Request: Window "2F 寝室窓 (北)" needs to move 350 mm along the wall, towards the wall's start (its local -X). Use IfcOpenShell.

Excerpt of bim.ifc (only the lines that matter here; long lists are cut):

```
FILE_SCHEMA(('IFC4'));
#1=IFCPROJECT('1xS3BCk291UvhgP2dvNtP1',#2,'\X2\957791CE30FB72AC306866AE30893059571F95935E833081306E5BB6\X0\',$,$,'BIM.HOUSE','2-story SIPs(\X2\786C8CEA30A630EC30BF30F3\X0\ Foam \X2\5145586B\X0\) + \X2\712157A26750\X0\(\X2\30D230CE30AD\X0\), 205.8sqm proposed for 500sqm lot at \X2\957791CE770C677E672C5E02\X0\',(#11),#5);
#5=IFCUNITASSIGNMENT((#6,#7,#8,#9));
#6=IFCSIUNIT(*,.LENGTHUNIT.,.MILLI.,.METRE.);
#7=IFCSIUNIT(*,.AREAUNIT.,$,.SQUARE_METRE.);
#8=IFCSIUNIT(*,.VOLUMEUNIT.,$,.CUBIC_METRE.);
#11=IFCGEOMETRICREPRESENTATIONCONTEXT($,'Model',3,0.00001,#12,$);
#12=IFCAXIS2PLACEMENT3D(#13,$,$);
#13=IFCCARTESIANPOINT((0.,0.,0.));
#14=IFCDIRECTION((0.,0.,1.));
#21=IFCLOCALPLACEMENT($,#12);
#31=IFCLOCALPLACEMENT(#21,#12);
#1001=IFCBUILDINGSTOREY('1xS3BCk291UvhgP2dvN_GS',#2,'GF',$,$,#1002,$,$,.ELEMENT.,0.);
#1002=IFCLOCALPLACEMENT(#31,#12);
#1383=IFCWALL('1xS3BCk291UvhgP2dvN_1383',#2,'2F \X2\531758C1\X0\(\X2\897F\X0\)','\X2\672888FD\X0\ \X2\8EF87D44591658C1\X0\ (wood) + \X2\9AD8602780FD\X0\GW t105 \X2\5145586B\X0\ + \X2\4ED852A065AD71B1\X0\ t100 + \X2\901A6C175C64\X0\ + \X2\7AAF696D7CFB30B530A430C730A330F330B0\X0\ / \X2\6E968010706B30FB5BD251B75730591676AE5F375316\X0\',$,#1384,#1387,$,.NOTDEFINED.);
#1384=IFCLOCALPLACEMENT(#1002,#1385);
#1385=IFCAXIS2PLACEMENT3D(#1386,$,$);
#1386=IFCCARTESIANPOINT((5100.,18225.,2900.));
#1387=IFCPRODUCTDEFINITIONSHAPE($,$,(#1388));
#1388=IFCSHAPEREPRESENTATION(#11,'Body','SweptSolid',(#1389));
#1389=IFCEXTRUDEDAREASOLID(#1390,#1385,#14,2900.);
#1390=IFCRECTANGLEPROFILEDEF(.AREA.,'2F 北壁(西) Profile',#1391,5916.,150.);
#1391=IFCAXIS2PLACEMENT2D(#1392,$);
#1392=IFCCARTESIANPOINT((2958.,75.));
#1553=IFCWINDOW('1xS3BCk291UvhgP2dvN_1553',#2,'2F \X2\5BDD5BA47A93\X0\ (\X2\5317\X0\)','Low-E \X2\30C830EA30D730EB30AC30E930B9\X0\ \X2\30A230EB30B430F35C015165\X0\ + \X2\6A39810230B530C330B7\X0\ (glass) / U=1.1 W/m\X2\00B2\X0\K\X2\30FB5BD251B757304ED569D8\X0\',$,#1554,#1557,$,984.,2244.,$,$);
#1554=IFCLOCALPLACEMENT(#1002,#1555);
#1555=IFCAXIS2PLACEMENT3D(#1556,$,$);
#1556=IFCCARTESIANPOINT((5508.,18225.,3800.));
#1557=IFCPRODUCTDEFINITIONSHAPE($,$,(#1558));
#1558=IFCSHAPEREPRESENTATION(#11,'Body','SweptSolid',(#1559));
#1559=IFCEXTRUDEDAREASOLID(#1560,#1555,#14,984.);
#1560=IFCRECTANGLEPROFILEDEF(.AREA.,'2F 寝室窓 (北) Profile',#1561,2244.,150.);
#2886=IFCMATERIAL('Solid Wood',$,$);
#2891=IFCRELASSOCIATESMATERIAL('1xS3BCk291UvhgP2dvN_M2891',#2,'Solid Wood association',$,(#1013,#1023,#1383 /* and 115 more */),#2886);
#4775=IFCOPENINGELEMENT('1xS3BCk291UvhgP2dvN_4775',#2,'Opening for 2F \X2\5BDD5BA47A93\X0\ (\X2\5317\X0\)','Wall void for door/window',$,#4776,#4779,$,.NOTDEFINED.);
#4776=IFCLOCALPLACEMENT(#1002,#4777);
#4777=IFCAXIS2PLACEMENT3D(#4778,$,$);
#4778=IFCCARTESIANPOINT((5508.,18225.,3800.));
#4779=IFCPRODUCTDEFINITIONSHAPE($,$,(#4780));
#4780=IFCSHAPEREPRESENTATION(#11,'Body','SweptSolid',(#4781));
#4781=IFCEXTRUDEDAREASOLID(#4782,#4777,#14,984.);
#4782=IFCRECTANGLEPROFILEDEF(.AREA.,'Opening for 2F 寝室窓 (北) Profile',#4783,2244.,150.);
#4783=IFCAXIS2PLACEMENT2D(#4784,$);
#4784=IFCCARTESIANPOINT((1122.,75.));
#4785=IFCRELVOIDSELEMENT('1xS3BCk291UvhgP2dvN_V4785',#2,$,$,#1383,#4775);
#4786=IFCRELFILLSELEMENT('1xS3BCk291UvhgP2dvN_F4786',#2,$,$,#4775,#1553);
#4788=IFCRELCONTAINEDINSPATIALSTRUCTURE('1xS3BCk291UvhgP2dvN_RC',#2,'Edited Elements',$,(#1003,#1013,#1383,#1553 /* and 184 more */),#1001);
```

```python
import ifcopenshell
import ifcopenshell.api.geometry
import ifcopenshell.util.placement
import ifcopenshell.util.unit

model = ifcopenshell.open("bim.ifc")
unit_scale = ifcopenshell.util.unit.calculate_unit_scale(model)

window = model.by_id(1553)
opening = window.FillsVoids[0].RelatingOpeningElement
wall = opening.VoidsElements[0].RelatingBuildingElement

wall_matrix = ifcopenshell.util.placement.get_local_placement(wall.ObjectPlacement)
shift = wall_matrix[:3, 0] * -0.35 / unit_scale
before = ifcopenshell.util.placement.get_local_placement(window.ObjectPlacement)[:3, 3].copy()

# The window is not placed relative to its opening, so move both.
for product in (opening, window):
    matrix = ifcopenshell.util.placement.get_local_placement(product.ObjectPlacement)
    matrix[:3, 3] += shift
    ifcopenshell.api.geometry.edit_object_placement(model, product=product, matrix=matrix, is_si=False)

after = ifcopenshell.util.placement.get_local_placement(window.ObjectPlacement)[:3, 3]
print("window moved by", (after - before).round(3) + 0.0)

model.write("bim_rev.ifc")
```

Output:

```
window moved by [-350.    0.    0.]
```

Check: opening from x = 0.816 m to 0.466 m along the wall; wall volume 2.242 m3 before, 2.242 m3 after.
